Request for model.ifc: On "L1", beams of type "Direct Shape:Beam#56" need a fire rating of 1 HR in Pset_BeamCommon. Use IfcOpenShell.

First a look at what the model holds.

```python
import ifcopenshell
import ifcopenshell.util.element

model = ifcopenshell.open("model.ifc")
print(model.schema)
storey = next(s for s in model.by_type("IfcBuildingStorey") if s.Name == "L1")
beams = [e for e in ifcopenshell.util.element.get_decomposition(storey) if e.is_a("IfcBeam")]
seen = {}
for e in beams:
    element_type = ifcopenshell.util.element.get_type(e)
    key = (element_type.Name if element_type != e and element_type else None, ifcopenshell.util.element.get_pset(e, "Pset_BeamCommon", "FireRating"))
    seen[key] = seen.get(key, 0) + 1
for (name, value), count in sorted(seen.items(), key=str):
    print(count, "x", name, "|", value)
```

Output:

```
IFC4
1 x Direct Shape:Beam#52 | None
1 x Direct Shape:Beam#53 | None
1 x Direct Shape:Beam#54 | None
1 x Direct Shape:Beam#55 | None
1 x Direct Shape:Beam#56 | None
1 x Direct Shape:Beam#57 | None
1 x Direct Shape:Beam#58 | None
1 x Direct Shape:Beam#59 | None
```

```python
import ifcopenshell
import ifcopenshell.api.pset
import ifcopenshell.util.element

model = ifcopenshell.open("model.ifc")

storey = next(s for s in model.by_type("IfcBuildingStorey") if s.Name == "L1")
beams = [e for e in ifcopenshell.util.element.get_decomposition(storey) if e.is_a("IfcBeam")]

count = 0
for e in beams:
    element_type = ifcopenshell.util.element.get_type(e)
    if element_type in (None, e) or element_type.Name != "Direct Shape:Beam#56":
        continue
    # add_pset returns the element's existing set when there is one.
    pset = ifcopenshell.api.pset.add_pset(model, product=e, name="Pset_BeamCommon")
    ifcopenshell.api.pset.edit_pset(model, pset=pset, properties={"FireRating": "1 HR"})
    count += 1

print(count, "beams updated")

model.write("model_v2.ifc")
```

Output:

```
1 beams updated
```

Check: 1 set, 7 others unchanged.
